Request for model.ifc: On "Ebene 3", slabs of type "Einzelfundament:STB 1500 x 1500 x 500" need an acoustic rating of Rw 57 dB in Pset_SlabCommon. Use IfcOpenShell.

First a look at what the model holds.

```python
import ifcopenshell
import ifcopenshell.util.element

model = ifcopenshell.open("model.ifc")
print(model.schema)
storey = next(s for s in model.by_type("IfcBuildingStorey") if s.Name == "Ebene 3")
slabs = [e for e in ifcopenshell.util.element.get_decomposition(storey) if e.is_a("IfcSlab")]
seen = {}
for e in slabs:
    element_type = ifcopenshell.util.element.get_type(e)
    key = (element_type.Name if element_type != e and element_type else None, ifcopenshell.util.element.get_pset(e, "Pset_SlabCommon", "AcousticRating"))
    seen[key] = seen.get(key, 0) + 1
for (name, value), count in sorted(seen.items(), key=str):
    print(count, "x", name, "|", value)
```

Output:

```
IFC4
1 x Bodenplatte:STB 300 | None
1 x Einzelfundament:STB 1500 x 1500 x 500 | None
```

```python
import ifcopenshell
import ifcopenshell.api.pset
import ifcopenshell.util.element

model = ifcopenshell.open("model.ifc")

storey = next(s for s in model.by_type("IfcBuildingStorey") if s.Name == "Ebene 3")
slabs = [e for e in ifcopenshell.util.element.get_decomposition(storey) if e.is_a("IfcSlab")]

count = 0
for e in slabs:
    element_type = ifcopenshell.util.element.get_type(e)
    if element_type in (None, e) or element_type.Name != "Einzelfundament:STB 1500 x 1500 x 500":
        continue
    # add_pset returns the element's existing set when there is one.
    pset = ifcopenshell.api.pset.add_pset(model, product=e, name="Pset_SlabCommon")
    ifcopenshell.api.pset.edit_pset(model, pset=pset, properties={"AcousticRating": "Rw 57 dB"})
    count += 1

print(count, "slabs updated")

model.write("model_rev.ifc")
```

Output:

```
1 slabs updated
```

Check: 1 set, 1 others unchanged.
